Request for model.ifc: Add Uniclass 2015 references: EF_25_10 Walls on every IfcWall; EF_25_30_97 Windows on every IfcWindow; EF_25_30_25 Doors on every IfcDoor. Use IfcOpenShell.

First a look at what the model holds.

```python
import ifcopenshell

model = ifcopenshell.open("model.ifc")
print(model.schema)
print("classifications:", [c.Name for c in model.by_type("IfcClassification")])
for ifc_class in ("IfcDoor", "IfcRoof", "IfcStair", "IfcWall", "IfcWindow"):
    print(ifc_class, len(model.by_type(ifc_class)))
```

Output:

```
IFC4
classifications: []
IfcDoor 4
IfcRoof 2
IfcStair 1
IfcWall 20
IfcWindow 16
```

```python
import ifcopenshell
import ifcopenshell.api.classification

model = ifcopenshell.open("model.ifc")

system = ifcopenshell.api.classification.add_classification(model, classification="Uniclass 2015")

codes = {
    "IfcWall": ("EF_25_10", "Walls"),
    "IfcWindow": ("EF_25_30_97", "Windows"),
    "IfcDoor": ("EF_25_30_25", "Doors"),
}
for ifc_class, (code, name) in codes.items():
    products = model.by_type(ifc_class)
    ifcopenshell.api.classification.add_reference(
        model, products=products, classification=system, identification=code, name=name
    )
    print(code, len(products))

model.write("model_edited.ifc")
```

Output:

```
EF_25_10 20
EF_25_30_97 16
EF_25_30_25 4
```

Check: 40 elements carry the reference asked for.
